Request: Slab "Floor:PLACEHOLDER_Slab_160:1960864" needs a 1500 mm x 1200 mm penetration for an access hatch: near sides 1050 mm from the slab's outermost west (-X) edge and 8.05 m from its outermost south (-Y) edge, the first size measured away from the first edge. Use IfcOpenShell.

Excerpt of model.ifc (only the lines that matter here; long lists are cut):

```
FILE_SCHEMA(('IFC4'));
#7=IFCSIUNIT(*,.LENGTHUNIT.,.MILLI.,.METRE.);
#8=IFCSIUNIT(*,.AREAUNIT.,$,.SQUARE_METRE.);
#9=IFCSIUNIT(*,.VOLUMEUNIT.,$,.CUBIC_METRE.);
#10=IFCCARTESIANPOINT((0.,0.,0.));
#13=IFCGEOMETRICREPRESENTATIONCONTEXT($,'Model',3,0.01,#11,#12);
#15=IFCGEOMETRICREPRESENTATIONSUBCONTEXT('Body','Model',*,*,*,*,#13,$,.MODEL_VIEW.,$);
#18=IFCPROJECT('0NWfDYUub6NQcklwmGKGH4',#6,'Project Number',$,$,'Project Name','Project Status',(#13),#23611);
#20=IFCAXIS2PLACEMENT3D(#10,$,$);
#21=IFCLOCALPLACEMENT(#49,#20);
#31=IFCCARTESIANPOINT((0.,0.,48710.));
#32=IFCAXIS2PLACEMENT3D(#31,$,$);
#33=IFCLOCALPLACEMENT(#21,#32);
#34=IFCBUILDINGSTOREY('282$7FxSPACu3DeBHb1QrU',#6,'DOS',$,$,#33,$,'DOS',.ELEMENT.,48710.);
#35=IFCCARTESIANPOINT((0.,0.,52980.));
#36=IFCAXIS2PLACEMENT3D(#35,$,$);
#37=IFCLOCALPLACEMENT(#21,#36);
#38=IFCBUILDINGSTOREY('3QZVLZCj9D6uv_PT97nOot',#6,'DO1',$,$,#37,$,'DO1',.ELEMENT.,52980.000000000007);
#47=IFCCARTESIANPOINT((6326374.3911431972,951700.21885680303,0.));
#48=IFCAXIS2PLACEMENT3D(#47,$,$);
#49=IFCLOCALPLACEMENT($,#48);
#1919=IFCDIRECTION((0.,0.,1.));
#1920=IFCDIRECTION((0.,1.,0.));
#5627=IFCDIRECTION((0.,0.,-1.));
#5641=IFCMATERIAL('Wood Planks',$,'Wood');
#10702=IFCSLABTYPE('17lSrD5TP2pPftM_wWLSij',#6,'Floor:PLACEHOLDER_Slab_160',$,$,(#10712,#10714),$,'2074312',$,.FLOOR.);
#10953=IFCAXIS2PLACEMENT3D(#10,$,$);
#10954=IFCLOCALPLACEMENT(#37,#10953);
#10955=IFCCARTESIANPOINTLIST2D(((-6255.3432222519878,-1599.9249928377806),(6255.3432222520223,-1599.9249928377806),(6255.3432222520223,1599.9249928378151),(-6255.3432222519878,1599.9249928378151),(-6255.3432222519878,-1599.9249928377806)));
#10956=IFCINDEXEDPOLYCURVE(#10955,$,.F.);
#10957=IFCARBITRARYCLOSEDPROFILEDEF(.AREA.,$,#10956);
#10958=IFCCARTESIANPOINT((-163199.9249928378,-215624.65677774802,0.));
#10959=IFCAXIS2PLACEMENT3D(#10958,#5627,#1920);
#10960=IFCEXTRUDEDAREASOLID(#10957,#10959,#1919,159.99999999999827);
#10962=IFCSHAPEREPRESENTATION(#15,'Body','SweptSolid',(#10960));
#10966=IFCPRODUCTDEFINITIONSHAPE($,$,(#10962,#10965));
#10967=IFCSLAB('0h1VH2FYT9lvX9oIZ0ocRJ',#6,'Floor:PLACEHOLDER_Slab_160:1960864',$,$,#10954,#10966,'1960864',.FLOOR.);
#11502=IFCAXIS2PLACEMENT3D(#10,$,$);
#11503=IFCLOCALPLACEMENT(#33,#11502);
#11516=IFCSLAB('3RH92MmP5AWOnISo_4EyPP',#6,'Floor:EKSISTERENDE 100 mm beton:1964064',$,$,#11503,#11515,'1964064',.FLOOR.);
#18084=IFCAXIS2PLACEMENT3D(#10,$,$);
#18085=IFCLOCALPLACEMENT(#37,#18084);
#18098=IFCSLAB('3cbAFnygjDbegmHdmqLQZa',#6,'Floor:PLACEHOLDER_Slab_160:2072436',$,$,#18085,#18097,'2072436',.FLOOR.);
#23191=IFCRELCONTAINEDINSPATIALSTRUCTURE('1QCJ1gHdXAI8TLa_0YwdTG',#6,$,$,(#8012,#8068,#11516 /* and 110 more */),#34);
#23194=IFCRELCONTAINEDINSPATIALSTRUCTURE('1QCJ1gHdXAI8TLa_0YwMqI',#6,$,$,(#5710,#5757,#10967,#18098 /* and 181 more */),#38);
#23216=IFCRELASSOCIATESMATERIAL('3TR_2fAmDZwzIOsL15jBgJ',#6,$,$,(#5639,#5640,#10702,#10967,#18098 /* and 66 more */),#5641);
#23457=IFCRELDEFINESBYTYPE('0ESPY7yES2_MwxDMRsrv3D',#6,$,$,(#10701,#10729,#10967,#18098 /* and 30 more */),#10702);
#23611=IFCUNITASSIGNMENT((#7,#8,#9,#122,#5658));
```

```python
import numpy as np
import ifcopenshell
import ifcopenshell.api.feature
import ifcopenshell.api.geometry
import ifcopenshell.api.root
import ifcopenshell.geom
import ifcopenshell.util.placement
import ifcopenshell.util.representation
import ifcopenshell.util.shape
import ifcopenshell.util.unit

model = ifcopenshell.open("model.ifc")
unit_scale = ifcopenshell.util.unit.calculate_unit_scale(model)
settings = ifcopenshell.geom.settings()


def volume(element):
    """Net volume in cubic metres, openings subtracted."""
    shape = ifcopenshell.geom.create_shape(settings, element)
    return ifcopenshell.util.shape.get_volume(shape.geometry)


slab = model.by_guid("0h1VH2FYT9lvX9oIZ0ocRJ")
before = volume(slab)

# Extent in the slab's own axes, in metres. The edges named are its -X and -Y sides.
slab_shape = ifcopenshell.geom.create_shape(settings, slab)
vertices = ifcopenshell.util.shape.get_vertices(slab_shape.geometry)
x_min, y_min, bottom = vertices.min(axis=0)
top = vertices[:, 2].max()

opening = ifcopenshell.api.root.create_entity(model, ifc_class="IfcOpeningElement", name="Access hatch opening", predefined_type="OPENING")
context = ifcopenshell.util.representation.get_context(model, "Model", "Body", "MODEL_VIEW")
width, depth = 1.5, 1.2
outline = [(0.0, 0.0), (width, 0.0), (width, depth), (0.0, depth), (0.0, 0.0)]
# Overshoot both faces by 50 mm so the cut is clean.
shape = ifcopenshell.api.geometry.add_slab_representation(
    model, context=context, depth=top - bottom + 0.1, polyline=outline
)
ifcopenshell.api.geometry.assign_representation(model, product=opening, representation=shape)

matrix = ifcopenshell.util.placement.get_local_placement(slab.ObjectPlacement)
matrix[:, 3] = matrix @ np.append(np.array([x_min + 1.05, y_min + 8.05, bottom - 0.05]) / unit_scale, 1.0)
ifcopenshell.api.geometry.edit_object_placement(model, product=opening, matrix=matrix, is_si=False)
ifcopenshell.api.feature.add_feature(model, feature=opening, element=slab)

after = volume(slab)

print(f"slab volume {before:.3f} -> {after:.3f} m3")

model.write("model-out.ifc")
```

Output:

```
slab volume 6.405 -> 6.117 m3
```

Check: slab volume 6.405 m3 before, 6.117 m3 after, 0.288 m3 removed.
